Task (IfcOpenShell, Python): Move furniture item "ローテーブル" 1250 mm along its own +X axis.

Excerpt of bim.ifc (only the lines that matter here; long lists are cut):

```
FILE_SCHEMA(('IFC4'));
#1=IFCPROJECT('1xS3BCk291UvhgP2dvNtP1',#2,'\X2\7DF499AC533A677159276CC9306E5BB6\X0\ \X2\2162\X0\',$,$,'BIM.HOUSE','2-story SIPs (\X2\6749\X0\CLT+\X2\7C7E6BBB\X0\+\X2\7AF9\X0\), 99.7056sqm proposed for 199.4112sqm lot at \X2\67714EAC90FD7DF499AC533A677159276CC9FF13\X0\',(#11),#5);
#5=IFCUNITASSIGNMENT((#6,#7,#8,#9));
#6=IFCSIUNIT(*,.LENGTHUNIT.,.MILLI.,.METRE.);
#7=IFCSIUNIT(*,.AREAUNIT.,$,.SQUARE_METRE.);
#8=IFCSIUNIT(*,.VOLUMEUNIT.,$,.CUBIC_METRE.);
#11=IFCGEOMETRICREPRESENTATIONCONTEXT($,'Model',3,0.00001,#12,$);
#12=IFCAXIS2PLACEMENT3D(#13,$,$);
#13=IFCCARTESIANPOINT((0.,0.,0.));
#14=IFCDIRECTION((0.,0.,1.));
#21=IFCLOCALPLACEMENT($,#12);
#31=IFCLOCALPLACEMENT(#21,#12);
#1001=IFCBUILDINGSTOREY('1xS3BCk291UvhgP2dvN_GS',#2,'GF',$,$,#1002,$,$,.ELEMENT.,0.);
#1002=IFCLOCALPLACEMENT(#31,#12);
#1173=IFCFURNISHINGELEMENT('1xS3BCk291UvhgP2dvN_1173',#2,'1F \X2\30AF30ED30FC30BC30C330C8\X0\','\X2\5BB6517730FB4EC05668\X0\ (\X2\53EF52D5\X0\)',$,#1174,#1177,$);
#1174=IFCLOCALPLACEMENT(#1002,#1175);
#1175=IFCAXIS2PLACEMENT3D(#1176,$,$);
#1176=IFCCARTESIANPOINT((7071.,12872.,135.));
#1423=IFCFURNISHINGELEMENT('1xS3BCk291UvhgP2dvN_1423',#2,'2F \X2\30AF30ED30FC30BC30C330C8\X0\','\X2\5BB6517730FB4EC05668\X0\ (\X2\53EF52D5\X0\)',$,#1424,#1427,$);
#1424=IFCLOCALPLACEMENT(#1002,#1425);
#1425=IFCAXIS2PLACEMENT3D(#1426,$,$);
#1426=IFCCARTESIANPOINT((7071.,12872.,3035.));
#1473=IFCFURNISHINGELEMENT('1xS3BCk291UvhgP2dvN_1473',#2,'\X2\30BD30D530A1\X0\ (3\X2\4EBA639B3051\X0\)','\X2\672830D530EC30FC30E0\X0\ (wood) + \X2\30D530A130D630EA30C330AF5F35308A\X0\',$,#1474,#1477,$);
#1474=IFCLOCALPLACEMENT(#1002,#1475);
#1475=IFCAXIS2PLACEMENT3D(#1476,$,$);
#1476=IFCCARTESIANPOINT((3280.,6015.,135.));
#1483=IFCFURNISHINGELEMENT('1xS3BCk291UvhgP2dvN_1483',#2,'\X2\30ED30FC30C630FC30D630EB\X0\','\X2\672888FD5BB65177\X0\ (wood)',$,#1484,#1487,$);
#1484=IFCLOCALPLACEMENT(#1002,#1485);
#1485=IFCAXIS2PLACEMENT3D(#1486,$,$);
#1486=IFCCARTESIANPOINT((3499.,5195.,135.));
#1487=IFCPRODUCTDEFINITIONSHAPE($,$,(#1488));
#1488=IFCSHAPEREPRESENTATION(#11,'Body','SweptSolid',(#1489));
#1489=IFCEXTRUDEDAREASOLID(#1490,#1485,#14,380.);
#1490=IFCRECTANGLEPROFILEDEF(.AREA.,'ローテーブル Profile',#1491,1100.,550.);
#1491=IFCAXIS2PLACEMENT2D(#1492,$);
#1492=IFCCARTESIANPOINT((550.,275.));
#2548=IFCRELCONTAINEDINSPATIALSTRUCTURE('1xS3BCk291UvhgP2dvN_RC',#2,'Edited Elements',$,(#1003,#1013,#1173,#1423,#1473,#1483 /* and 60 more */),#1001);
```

```python
import ifcopenshell
import ifcopenshell.api.geometry
import ifcopenshell.util.placement
import ifcopenshell.util.unit

model = ifcopenshell.open("bim.ifc")
unit_scale = ifcopenshell.util.unit.calculate_unit_scale(model)

item = model.by_guid("1xS3BCk291UvhgP2dvN_1483")
matrix = ifcopenshell.util.placement.get_local_placement(item.ObjectPlacement)
matrix[:3, 3] += matrix[:3, 0] * 1.25 / unit_scale
ifcopenshell.api.geometry.edit_object_placement(model, product=item, matrix=matrix, is_si=False)

print(ifcopenshell.util.placement.get_local_placement(item.ObjectPlacement).round(3) + 0.0)

model.write("bim_rev.ifc")
```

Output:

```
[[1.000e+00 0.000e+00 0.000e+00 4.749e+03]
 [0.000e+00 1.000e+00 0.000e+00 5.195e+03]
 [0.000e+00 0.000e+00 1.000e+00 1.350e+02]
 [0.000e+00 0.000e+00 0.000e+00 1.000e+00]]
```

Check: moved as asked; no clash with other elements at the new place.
